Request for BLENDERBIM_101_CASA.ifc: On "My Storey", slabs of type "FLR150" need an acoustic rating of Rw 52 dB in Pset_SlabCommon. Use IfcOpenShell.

First a look at what the model holds.

```python
import ifcopenshell
import ifcopenshell.util.element

model = ifcopenshell.open("BLENDERBIM_101_CASA.ifc")
print(model.schema)
storey = next(s for s in model.by_type("IfcBuildingStorey") if s.Name == "My Storey")
slabs = [e for e in ifcopenshell.util.element.get_decomposition(storey) if e.is_a("IfcSlab")]
seen = {}
for e in slabs:
    element_type = ifcopenshell.util.element.get_type(e)
    key = (element_type.Name if element_type != e and element_type else None, ifcopenshell.util.element.get_pset(e, "Pset_SlabCommon", "AcousticRating"))
    seen[key] = seen.get(key, 0) + 1
for (name, value), count in sorted(seen.items(), key=str):
    print(count, "x", name, "|", value)
```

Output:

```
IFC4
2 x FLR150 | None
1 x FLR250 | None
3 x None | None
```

```python
import ifcopenshell
import ifcopenshell.api.pset
import ifcopenshell.util.element

model = ifcopenshell.open("BLENDERBIM_101_CASA.ifc")

storey = next(s for s in model.by_type("IfcBuildingStorey") if s.Name == "My Storey")
slabs = [e for e in ifcopenshell.util.element.get_decomposition(storey) if e.is_a("IfcSlab")]

count = 0
for e in slabs:
    element_type = ifcopenshell.util.element.get_type(e)
    if element_type in (None, e) or element_type.Name != "FLR150":
        continue
    # add_pset returns the element's existing set when there is one.
    pset = ifcopenshell.api.pset.add_pset(model, product=e, name="Pset_SlabCommon")
    ifcopenshell.api.pset.edit_pset(model, pset=pset, properties={"AcousticRating": "Rw 52 dB"})
    count += 1

print(count, "slabs updated")

model.write("BLENDERBIM_101_CASA_updated.ifc")
```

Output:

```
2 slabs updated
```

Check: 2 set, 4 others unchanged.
